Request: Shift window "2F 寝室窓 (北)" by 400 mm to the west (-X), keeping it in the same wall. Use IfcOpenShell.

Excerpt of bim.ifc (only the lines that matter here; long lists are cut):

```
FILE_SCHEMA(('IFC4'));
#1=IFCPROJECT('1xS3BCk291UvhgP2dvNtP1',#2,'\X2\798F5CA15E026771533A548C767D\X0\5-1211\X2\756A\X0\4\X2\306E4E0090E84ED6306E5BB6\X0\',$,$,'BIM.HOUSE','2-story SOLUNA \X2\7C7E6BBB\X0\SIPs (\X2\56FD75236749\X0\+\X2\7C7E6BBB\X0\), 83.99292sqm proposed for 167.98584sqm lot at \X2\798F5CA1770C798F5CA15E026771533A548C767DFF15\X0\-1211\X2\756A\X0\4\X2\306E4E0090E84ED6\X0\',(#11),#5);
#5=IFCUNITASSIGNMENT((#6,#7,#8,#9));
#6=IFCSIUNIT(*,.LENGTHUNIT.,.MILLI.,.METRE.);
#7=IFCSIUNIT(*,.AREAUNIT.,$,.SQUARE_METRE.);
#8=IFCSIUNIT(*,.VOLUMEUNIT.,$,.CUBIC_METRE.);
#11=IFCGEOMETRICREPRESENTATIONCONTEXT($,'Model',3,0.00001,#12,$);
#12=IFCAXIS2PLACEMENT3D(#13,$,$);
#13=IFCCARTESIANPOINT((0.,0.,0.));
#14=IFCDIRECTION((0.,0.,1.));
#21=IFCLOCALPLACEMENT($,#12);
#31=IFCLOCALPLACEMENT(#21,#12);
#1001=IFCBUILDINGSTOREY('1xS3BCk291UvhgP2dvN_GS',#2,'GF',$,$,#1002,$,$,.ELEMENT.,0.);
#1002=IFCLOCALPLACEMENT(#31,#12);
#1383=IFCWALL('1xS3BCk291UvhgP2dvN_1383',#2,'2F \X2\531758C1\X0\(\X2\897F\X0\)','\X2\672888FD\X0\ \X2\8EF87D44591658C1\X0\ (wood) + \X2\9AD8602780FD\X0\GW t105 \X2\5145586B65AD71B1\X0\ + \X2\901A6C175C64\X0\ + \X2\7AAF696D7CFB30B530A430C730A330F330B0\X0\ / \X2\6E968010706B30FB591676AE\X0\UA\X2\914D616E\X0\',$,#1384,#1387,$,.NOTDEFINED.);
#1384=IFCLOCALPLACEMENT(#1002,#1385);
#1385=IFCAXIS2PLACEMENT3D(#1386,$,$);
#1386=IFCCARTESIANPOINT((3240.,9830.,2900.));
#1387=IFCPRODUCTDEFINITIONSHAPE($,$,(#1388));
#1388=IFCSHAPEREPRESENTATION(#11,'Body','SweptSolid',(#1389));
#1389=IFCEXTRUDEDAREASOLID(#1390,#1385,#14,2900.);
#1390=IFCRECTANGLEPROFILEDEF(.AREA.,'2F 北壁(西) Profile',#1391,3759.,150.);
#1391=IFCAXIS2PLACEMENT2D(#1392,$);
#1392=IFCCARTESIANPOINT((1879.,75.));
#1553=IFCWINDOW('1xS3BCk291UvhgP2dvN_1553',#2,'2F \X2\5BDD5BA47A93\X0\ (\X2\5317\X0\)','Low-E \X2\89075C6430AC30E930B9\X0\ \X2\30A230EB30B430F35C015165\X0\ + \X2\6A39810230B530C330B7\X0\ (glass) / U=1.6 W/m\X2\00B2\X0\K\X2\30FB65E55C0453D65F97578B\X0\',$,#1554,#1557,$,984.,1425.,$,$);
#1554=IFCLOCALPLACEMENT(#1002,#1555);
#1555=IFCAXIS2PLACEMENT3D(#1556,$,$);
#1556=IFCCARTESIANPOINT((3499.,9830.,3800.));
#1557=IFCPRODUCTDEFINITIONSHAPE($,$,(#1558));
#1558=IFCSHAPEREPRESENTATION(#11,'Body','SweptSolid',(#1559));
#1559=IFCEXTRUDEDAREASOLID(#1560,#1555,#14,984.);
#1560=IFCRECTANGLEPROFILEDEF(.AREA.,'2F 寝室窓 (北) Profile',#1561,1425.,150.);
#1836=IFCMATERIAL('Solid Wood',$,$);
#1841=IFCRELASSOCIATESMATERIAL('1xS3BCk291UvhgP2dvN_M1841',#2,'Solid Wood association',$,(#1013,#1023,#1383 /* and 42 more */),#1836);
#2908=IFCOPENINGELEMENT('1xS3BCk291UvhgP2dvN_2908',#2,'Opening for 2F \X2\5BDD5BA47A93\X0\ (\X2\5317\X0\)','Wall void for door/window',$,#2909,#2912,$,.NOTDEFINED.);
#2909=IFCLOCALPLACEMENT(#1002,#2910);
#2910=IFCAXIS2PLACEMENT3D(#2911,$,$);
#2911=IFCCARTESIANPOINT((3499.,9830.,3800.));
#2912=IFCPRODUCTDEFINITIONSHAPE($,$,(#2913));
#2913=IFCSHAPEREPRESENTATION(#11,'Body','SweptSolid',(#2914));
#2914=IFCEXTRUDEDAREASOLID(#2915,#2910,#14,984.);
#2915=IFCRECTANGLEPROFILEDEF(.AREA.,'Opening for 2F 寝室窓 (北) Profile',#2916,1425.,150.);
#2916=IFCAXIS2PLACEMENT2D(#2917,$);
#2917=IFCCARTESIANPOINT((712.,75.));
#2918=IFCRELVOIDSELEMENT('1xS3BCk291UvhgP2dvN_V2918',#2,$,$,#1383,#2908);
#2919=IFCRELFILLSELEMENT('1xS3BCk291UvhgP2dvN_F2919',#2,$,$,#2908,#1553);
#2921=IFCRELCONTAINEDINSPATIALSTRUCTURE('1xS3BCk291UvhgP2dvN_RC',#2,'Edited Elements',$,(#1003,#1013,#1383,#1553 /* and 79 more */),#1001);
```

```python
import ifcopenshell
import ifcopenshell.api.geometry
import ifcopenshell.util.placement
import ifcopenshell.util.unit

model = ifcopenshell.open("bim.ifc")
unit_scale = ifcopenshell.util.unit.calculate_unit_scale(model)

window = model.by_guid("1xS3BCk291UvhgP2dvN_1553")
opening = window.FillsVoids[0].RelatingOpeningElement
wall = opening.VoidsElements[0].RelatingBuildingElement

wall_matrix = ifcopenshell.util.placement.get_local_placement(wall.ObjectPlacement)
shift = wall_matrix[:3, 0] * -0.4 / unit_scale
before = ifcopenshell.util.placement.get_local_placement(window.ObjectPlacement)[:3, 3].copy()

# The window is not placed relative to its opening, so move both.
for product in (opening, window):
    matrix = ifcopenshell.util.placement.get_local_placement(product.ObjectPlacement)
    matrix[:3, 3] += shift
    ifcopenshell.api.geometry.edit_object_placement(model, product=product, matrix=matrix, is_si=False)

after = ifcopenshell.util.placement.get_local_placement(window.ObjectPlacement)[:3, 3]
print("window moved by", (after - before).round(3) + 0.0)

model.write("bim-out.ifc")
```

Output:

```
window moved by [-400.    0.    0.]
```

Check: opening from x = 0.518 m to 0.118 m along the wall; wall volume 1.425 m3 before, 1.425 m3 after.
